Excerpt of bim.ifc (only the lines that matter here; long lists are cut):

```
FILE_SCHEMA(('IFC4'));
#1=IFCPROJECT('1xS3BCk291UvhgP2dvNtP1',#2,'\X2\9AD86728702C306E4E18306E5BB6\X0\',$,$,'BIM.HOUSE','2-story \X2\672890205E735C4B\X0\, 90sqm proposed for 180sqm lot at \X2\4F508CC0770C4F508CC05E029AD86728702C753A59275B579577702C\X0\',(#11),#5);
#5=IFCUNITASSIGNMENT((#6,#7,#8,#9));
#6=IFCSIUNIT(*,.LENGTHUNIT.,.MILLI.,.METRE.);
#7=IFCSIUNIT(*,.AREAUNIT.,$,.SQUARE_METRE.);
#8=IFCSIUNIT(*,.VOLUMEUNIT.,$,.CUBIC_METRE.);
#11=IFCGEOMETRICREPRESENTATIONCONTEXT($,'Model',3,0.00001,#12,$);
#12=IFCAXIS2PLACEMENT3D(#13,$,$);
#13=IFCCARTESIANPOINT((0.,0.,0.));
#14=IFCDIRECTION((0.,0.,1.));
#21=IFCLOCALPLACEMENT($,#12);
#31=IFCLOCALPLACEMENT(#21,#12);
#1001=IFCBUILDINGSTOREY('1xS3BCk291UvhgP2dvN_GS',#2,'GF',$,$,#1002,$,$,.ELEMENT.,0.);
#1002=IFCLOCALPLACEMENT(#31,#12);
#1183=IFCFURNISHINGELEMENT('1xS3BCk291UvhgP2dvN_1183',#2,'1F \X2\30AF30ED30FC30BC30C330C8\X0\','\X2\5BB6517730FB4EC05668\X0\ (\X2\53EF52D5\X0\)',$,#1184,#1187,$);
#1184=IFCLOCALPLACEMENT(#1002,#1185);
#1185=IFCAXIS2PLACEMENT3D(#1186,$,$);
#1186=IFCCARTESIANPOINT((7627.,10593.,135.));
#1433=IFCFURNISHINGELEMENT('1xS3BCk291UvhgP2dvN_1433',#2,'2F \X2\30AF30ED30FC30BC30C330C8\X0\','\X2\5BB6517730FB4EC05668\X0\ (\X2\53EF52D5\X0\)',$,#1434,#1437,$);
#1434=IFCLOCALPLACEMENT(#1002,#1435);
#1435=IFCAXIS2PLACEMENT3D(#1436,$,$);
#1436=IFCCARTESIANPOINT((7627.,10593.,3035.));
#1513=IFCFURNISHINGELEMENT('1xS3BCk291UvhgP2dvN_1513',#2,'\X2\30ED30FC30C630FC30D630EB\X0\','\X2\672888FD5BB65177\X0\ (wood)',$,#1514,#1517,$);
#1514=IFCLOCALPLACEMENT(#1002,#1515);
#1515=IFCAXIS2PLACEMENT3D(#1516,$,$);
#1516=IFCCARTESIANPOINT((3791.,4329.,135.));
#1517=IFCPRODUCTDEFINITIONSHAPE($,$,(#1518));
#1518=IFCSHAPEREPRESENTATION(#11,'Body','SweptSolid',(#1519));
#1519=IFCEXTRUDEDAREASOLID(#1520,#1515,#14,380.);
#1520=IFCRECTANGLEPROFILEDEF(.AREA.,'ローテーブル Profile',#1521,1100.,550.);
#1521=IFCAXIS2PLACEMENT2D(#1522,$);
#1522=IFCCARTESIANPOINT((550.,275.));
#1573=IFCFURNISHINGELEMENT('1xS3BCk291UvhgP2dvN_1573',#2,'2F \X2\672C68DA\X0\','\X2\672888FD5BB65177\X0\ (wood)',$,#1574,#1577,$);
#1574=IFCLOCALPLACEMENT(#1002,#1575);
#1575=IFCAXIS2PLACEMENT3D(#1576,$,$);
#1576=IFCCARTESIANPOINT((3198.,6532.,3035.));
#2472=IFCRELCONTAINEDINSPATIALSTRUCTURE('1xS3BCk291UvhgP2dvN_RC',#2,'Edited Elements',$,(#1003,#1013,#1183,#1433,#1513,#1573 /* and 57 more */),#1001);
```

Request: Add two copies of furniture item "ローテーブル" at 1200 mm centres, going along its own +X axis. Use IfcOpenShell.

```python
import ifcopenshell
import ifcopenshell.api.geometry
import ifcopenshell.api.root
import ifcopenshell.util.element
import ifcopenshell.util.placement
import ifcopenshell.util.unit

model = ifcopenshell.open("bim.ifc")
unit_scale = ifcopenshell.util.unit.calculate_unit_scale(model)


def reuse_history(source, copy):
    """copy_class also copies each property set's owner history, people and application; keep the originals."""
    for rel in copy.IsDefinedBy:
        if rel.is_a("IfcRelDefinesByProperties") and (history := rel.RelatingPropertyDefinition.OwnerHistory):
            rel.RelatingPropertyDefinition.OwnerHistory = source.OwnerHistory
            ifcopenshell.util.element.remove_deep2(model, history)


source = model.by_guid("1xS3BCk291UvhgP2dvN_1513")
base = ifcopenshell.util.placement.get_local_placement(source.ObjectPlacement)
step = base[:3, 0] * 1.2 / unit_scale

for i in range(1, 3):
    copy = ifcopenshell.api.root.copy_class(model, product=source)
    copy.Representation = ifcopenshell.util.element.copy_deep(
        model, source.Representation, exclude=["IfcGeometricRepresentationContext", "IfcRepresentationMap"]
    )
    reuse_history(source, copy)
    matrix = base.copy()
    matrix[:3, 3] += i * step
    print("added at", matrix[:3, 3].round(3) + 0.0)
    ifcopenshell.api.geometry.edit_object_placement(model, product=copy, matrix=matrix, is_si=False)

model.write("bim_rev.ifc")
```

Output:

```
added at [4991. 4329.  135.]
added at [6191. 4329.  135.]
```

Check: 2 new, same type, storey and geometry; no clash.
